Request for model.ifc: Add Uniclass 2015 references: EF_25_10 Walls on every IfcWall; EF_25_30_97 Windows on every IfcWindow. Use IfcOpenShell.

First a look at what the model holds.

```python
import ifcopenshell

model = ifcopenshell.open("model.ifc")
print(model.schema)
print("classifications:", [c.Name for c in model.by_type("IfcClassification")])
for ifc_class in ("IfcDoor", "IfcRoof", "IfcStair", "IfcWall", "IfcWindow"):
    print(ifc_class, len(model.by_type(ifc_class)))
```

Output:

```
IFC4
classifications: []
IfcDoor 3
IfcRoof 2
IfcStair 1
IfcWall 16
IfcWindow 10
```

```python
import ifcopenshell
import ifcopenshell.api.classification

model = ifcopenshell.open("model.ifc")

system = ifcopenshell.api.classification.add_classification(model, classification="Uniclass 2015")

codes = {
    "IfcWall": ("EF_25_10", "Walls"),
    "IfcWindow": ("EF_25_30_97", "Windows"),
}
for ifc_class, (code, name) in codes.items():
    products = model.by_type(ifc_class)
    ifcopenshell.api.classification.add_reference(
        model, products=products, classification=system, identification=code, name=name
    )
    print(code, len(products))

model.write("model_edited.ifc")
```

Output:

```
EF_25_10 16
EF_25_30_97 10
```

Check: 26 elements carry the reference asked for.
